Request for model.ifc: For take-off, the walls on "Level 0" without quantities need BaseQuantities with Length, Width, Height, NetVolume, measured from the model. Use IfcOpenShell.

First a look at what the model holds.

```python
import ifcopenshell
import ifcopenshell.util.element
import ifcopenshell.util.unit

model = ifcopenshell.open("model.ifc")
print(model.schema)
for unit_type in ("LENGTHUNIT", "AREAUNIT", "VOLUMEUNIT"):
    print(unit_type, ifcopenshell.util.unit.calculate_unit_scale(model, unit_type))
storey = next(s for s in model.by_type("IfcBuildingStorey") if s.Name == "Level 0")
walls = [e for e in ifcopenshell.util.element.get_decomposition(storey) if e.is_a("IfcWall")]
for e in sorted(walls, key=lambda e: e.id()):
    print(e.id(), e.is_a(), e.Name, list(ifcopenshell.util.element.get_psets(e, qtos_only=True)), sep=" | ")
```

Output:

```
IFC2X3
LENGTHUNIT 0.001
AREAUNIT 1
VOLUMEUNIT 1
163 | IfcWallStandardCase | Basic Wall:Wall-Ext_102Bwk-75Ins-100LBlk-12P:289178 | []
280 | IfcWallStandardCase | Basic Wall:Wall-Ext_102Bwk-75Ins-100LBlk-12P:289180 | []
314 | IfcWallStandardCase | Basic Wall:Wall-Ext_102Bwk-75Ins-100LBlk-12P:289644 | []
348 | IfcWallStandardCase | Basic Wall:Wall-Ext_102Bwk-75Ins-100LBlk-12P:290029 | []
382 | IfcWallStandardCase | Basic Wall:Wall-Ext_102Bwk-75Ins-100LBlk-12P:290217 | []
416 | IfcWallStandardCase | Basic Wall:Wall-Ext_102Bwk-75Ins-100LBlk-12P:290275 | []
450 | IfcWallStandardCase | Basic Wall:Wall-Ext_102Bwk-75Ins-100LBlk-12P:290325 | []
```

```python
import ifcopenshell
import ifcopenshell.api.pset
import ifcopenshell.geom
import ifcopenshell.util.element
import ifcopenshell.util.shape
import ifcopenshell.util.unit

model = ifcopenshell.open("model.ifc")
unit_scale = ifcopenshell.util.unit.calculate_unit_scale(model)
volume_scale = ifcopenshell.util.unit.calculate_unit_scale(model, "VOLUMEUNIT")
settings = ifcopenshell.geom.settings()

storey = next(s for s in model.by_type("IfcBuildingStorey") if s.Name == "Level 0")
walls = [e for e in ifcopenshell.util.element.get_decomposition(storey) if e.is_a("IfcWall")]

for e in sorted(walls, key=lambda e: e.id()):
    if ifcopenshell.util.element.get_psets(e, qtos_only=True, should_inherit=False):
        continue
    # Geometry comes back in metres, in the element's own axes.
    shape = ifcopenshell.geom.create_shape(settings, e)
    values = {
        "Length": ifcopenshell.util.shape.get_x(shape.geometry) / unit_scale,
        "Width": ifcopenshell.util.shape.get_y(shape.geometry) / unit_scale,
        "Height": ifcopenshell.util.shape.get_z(shape.geometry) / unit_scale,
        "NetVolume": ifcopenshell.util.shape.get_volume(shape.geometry) / volume_scale,
    }
    qto = ifcopenshell.api.pset.add_qto(model, product=e, name="BaseQuantities")
    ifcopenshell.api.pset.edit_qto(model, qto=qto, properties=values)
    print(e.id(), {k: round(v, 3) for k, v in values.items()})

model.write("model-out.ifc")
```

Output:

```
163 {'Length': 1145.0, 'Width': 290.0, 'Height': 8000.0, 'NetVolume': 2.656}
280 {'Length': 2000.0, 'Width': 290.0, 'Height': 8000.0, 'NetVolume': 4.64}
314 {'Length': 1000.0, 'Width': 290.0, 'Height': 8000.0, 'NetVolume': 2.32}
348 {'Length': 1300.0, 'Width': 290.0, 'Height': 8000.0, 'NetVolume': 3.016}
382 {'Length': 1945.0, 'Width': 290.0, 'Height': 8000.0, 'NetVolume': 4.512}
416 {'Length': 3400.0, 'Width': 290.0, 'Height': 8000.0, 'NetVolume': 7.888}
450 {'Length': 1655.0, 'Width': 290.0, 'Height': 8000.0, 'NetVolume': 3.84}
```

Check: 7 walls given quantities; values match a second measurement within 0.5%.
